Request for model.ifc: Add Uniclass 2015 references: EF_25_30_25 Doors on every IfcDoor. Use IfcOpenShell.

First a look at what the model holds.

```python
import ifcopenshell

model = ifcopenshell.open("model.ifc")
print(model.schema)
print("classifications:", [c.Name for c in model.by_type("IfcClassification")])
for ifc_class in ("IfcDoor", "IfcRoof", "IfcStair", "IfcWall", "IfcWindow"):
    print(ifc_class, len(model.by_type(ifc_class)))
```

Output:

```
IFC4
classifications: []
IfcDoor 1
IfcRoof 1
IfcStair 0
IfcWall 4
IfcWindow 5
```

```python
import ifcopenshell
import ifcopenshell.api.classification

model = ifcopenshell.open("model.ifc")

system = ifcopenshell.api.classification.add_classification(model, classification="Uniclass 2015")

codes = {
    "IfcDoor": ("EF_25_30_25", "Doors"),
}
for ifc_class, (code, name) in codes.items():
    products = model.by_type(ifc_class)
    ifcopenshell.api.classification.add_reference(
        model, products=products, classification=system, identification=code, name=name
    )
    print(code, len(products))

model.write("model_updated.ifc")
```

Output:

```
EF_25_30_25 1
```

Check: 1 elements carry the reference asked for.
